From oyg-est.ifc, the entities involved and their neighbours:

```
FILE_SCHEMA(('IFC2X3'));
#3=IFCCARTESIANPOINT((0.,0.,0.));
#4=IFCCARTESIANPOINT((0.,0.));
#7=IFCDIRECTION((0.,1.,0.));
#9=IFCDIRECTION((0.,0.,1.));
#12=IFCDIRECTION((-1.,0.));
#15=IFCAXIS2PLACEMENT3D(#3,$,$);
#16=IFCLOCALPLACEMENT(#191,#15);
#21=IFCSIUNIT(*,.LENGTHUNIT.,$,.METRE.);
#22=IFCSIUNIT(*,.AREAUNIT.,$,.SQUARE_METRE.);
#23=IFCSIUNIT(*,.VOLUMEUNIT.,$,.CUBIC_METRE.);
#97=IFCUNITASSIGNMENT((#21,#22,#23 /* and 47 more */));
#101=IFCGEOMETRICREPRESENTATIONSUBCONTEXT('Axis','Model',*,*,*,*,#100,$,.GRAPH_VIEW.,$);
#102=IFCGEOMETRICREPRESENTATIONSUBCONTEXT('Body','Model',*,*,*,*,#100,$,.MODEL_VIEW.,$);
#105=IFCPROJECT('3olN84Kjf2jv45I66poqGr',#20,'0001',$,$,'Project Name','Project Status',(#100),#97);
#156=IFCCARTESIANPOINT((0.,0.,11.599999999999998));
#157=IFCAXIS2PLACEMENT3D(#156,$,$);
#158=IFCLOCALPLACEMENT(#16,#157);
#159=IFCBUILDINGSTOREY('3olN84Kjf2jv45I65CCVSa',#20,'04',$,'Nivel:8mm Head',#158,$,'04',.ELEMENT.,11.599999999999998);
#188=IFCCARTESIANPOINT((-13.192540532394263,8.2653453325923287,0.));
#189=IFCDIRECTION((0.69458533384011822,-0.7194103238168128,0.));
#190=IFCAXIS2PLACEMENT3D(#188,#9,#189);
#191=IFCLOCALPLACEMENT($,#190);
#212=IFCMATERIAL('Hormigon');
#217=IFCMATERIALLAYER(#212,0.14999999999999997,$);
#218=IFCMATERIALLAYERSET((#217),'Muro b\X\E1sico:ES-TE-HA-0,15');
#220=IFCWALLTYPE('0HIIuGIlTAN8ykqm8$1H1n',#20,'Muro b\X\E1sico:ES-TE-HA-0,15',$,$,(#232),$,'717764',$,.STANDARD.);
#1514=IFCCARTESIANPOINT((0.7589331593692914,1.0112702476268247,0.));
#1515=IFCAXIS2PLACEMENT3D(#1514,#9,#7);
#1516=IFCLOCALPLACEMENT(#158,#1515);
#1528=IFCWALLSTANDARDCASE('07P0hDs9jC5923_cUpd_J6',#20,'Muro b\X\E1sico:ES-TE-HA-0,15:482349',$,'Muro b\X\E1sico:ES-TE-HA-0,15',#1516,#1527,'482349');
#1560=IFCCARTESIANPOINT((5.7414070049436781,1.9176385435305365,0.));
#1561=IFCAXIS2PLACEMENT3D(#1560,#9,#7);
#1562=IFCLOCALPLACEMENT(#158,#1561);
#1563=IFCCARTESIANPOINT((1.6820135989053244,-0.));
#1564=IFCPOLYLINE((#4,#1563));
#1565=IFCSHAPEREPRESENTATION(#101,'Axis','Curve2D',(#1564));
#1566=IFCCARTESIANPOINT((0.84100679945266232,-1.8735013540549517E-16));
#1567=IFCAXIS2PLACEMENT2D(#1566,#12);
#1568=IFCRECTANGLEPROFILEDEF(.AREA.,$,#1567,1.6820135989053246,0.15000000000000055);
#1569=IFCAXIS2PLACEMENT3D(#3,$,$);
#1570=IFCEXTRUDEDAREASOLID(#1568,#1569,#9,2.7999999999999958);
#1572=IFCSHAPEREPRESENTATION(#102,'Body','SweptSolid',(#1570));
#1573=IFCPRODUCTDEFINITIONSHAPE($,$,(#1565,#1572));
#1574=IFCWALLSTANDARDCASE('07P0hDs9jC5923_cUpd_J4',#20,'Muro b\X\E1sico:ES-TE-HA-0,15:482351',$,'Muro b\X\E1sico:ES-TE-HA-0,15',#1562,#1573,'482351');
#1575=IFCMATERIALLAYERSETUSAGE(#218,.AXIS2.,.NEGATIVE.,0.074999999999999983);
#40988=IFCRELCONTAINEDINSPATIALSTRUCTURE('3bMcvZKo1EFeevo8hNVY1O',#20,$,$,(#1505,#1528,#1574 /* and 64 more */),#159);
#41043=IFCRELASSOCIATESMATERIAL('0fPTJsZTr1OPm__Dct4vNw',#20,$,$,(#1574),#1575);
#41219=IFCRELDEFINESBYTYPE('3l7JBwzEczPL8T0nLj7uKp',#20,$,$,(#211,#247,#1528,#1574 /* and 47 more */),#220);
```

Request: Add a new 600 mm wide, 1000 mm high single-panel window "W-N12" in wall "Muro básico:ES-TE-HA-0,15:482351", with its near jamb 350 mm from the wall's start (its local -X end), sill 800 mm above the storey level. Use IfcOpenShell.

```python
import numpy as np
import ifcopenshell
import ifcopenshell.api.feature
import ifcopenshell.api.geometry
import ifcopenshell.api.root
import ifcopenshell.api.spatial
import ifcopenshell.api.type
import ifcopenshell.geom
import ifcopenshell.util.element
import ifcopenshell.util.placement
import ifcopenshell.util.representation
import ifcopenshell.util.shape
import ifcopenshell.util.unit

model = ifcopenshell.open("oyg-est.ifc")
unit_scale = ifcopenshell.util.unit.calculate_unit_scale(model)
settings = ifcopenshell.geom.settings()


def volume(element):
    """Net volume in cubic metres, openings subtracted."""
    shape = ifcopenshell.geom.create_shape(settings, element)
    return ifcopenshell.util.shape.get_volume(shape.geometry)


wall = model.by_guid("07P0hDs9jC5923_cUpd_J4")
storey = ifcopenshell.util.element.get_container(wall, ifc_class="IfcBuildingStorey")
context = ifcopenshell.util.representation.get_context(model, "Model", "Body", "MODEL_VIEW")
before = volume(wall)

width, height, from_end, sill = 0.6, 1, 0.35, 0.8  # metres

# The wall runs along its own X axis, and the end named is its -X end.
wall_shape = ifcopenshell.geom.create_shape(settings, wall)
x, y, z = ifcopenshell.util.shape.get_vertices(wall_shape.geometry).T
start = x.min() + from_end
face, thickness = float(y.min()), float(y.max() - y.min())
wall_matrix = ifcopenshell.util.placement.get_local_placement(wall.ObjectPlacement)
level = ifcopenshell.util.placement.get_local_placement(storey.ObjectPlacement)[2, 3]


def in_wall(x, y):
    """Placement at x, y metres in the wall's axes, at sill height."""
    matrix = wall_matrix.copy()
    matrix[:, 3] = wall_matrix @ np.array([x / unit_scale, y / unit_scale, 0.0, 1.0])
    matrix[2, 3] = level + sill / unit_scale
    return matrix


# Opening: a box that overshoots both wall faces by 50 mm.
opening = ifcopenshell.api.root.create_entity(model, ifc_class="IfcOpeningElement")
box = ifcopenshell.api.geometry.add_wall_representation(
    model, context=context, length=width, height=height, thickness=thickness + 0.1
)
ifcopenshell.api.geometry.assign_representation(model, product=opening, representation=box)
ifcopenshell.api.geometry.edit_object_placement(model, product=opening, matrix=in_wall(start, face - 0.05), is_si=False)
ifcopenshell.api.feature.add_feature(model, feature=opening, element=wall)

window = ifcopenshell.api.root.create_entity(model, ifc_class="IfcWindow", name="W-N12")
window.OverallWidth, window.OverallHeight = width / unit_scale, height / unit_scale
body = ifcopenshell.api.geometry.add_window_representation(
    model,
    context=context,
    overall_width=window.OverallWidth,
    overall_height=window.OverallHeight,
    partition_type="SINGLE_PANEL",
)
ifcopenshell.api.geometry.assign_representation(model, product=window, representation=body)
ifcopenshell.api.spatial.assign_container(model, products=[window], relating_structure=storey)
fills = ifcopenshell.api.feature.add_filling(model, opening=opening, element=window)
fills.OwnerHistory = window.OwnerHistory  # required in IFC2X3

# IFC2X3 keeps the operation on the window style.
style = ifcopenshell.api.root.create_entity(model, ifc_class="IfcWindowStyle", name="W-N12")
style.OperationType, style.ConstructionType = "SINGLE_PANEL", "NOTDEFINED"
style.ParameterTakesPrecedence = style.Sizeable = False
ifcopenshell.api.type.assign_type(model, related_objects=[window], relating_type=style)

# Centre the window in the wall's thickness.
ifcopenshell.api.geometry.edit_object_placement(model, product=window, matrix=in_wall(start, face), is_si=False)
window_shape = ifcopenshell.geom.create_shape(settings, window)
depth = ifcopenshell.util.shape.get_vertices(window_shape.geometry)[:, 1]
offset = face + thickness / 2 - (depth.min() + depth.max()) / 2
ifcopenshell.api.geometry.edit_object_placement(model, product=window, matrix=in_wall(start, offset), is_si=False)

after = volume(wall)

print(f"wall volume {before:.3f} -> {after:.3f} m3")

model.write("oyg-est_edited.ifc")
```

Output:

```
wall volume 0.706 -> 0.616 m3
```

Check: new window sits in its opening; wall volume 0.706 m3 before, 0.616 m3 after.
